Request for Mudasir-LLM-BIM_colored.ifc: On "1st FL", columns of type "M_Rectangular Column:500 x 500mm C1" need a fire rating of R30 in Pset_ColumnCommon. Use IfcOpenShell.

First a look at what the model holds.

```python
import ifcopenshell
import ifcopenshell.util.element

model = ifcopenshell.open("Mudasir-LLM-BIM_colored.ifc")
print(model.schema)
storey = next(s for s in model.by_type("IfcBuildingStorey") if s.Name == "1st FL")
columns = [e for e in ifcopenshell.util.element.get_decomposition(storey) if e.is_a("IfcColumn")]
seen = {}
for e in columns:
    element_type = ifcopenshell.util.element.get_type(e)
    key = (element_type.Name if element_type != e and element_type else None, ifcopenshell.util.element.get_pset(e, "Pset_ColumnCommon", "FireRating"))
    seen[key] = seen.get(key, 0) + 1
for (name, value), count in sorted(seen.items(), key=str):
    print(count, "x", name, "|", value)
```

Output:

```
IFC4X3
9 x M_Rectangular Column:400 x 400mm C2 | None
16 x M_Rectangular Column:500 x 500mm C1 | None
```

```python
import ifcopenshell
import ifcopenshell.api.pset
import ifcopenshell.util.element

model = ifcopenshell.open("Mudasir-LLM-BIM_colored.ifc")

storey = next(s for s in model.by_type("IfcBuildingStorey") if s.Name == "1st FL")
columns = [e for e in ifcopenshell.util.element.get_decomposition(storey) if e.is_a("IfcColumn")]

count = 0
for e in columns:
    element_type = ifcopenshell.util.element.get_type(e)
    if element_type in (None, e) or element_type.Name != "M_Rectangular Column:500 x 500mm C1":
        continue
    # add_pset returns the element's existing set when there is one.
    pset = ifcopenshell.api.pset.add_pset(model, product=e, name="Pset_ColumnCommon")
    ifcopenshell.api.pset.edit_pset(model, pset=pset, properties={"FireRating": "R30"})
    count += 1

print(count, "columns updated")

model.write("Mudasir-LLM-BIM_colored_edited.ifc")
```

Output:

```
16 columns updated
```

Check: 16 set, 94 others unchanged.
